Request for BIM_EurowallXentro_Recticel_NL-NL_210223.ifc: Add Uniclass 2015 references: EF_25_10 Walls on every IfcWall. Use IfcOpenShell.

First a look at what the model holds.

```python
import ifcopenshell

model = ifcopenshell.open("BIM_EurowallXentro_Recticel_NL-NL_210223.ifc")
print(model.schema)
print("classifications:", [c.Name for c in model.by_type("IfcClassification")])
for ifc_class in ("IfcDoor", "IfcRoof", "IfcStair", "IfcWall", "IfcWindow"):
    print(ifc_class, len(model.by_type(ifc_class)))
```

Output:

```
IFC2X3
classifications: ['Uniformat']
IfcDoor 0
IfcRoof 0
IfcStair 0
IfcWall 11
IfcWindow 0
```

```python
import ifcopenshell
import ifcopenshell.api.classification

model = ifcopenshell.open("BIM_EurowallXentro_Recticel_NL-NL_210223.ifc")

# IFC2X3 requires Source and Edition and has no link from the project to the system.
system = model.create_entity("IfcClassification", Source="NBS", Edition="2015", Name="Uniclass 2015")

codes = {
    "IfcWall": ("EF_25_10", "Walls"),
}
for ifc_class, (code, name) in codes.items():
    products = model.by_type(ifc_class)
    ifcopenshell.api.classification.add_reference(
        model, products=products, classification=system, identification=code, name=name
    )
    print(code, len(products))

model.write("BIM_EurowallXentro_Recticel_NL-NL_210223_v2.ifc")
```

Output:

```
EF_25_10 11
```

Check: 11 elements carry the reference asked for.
